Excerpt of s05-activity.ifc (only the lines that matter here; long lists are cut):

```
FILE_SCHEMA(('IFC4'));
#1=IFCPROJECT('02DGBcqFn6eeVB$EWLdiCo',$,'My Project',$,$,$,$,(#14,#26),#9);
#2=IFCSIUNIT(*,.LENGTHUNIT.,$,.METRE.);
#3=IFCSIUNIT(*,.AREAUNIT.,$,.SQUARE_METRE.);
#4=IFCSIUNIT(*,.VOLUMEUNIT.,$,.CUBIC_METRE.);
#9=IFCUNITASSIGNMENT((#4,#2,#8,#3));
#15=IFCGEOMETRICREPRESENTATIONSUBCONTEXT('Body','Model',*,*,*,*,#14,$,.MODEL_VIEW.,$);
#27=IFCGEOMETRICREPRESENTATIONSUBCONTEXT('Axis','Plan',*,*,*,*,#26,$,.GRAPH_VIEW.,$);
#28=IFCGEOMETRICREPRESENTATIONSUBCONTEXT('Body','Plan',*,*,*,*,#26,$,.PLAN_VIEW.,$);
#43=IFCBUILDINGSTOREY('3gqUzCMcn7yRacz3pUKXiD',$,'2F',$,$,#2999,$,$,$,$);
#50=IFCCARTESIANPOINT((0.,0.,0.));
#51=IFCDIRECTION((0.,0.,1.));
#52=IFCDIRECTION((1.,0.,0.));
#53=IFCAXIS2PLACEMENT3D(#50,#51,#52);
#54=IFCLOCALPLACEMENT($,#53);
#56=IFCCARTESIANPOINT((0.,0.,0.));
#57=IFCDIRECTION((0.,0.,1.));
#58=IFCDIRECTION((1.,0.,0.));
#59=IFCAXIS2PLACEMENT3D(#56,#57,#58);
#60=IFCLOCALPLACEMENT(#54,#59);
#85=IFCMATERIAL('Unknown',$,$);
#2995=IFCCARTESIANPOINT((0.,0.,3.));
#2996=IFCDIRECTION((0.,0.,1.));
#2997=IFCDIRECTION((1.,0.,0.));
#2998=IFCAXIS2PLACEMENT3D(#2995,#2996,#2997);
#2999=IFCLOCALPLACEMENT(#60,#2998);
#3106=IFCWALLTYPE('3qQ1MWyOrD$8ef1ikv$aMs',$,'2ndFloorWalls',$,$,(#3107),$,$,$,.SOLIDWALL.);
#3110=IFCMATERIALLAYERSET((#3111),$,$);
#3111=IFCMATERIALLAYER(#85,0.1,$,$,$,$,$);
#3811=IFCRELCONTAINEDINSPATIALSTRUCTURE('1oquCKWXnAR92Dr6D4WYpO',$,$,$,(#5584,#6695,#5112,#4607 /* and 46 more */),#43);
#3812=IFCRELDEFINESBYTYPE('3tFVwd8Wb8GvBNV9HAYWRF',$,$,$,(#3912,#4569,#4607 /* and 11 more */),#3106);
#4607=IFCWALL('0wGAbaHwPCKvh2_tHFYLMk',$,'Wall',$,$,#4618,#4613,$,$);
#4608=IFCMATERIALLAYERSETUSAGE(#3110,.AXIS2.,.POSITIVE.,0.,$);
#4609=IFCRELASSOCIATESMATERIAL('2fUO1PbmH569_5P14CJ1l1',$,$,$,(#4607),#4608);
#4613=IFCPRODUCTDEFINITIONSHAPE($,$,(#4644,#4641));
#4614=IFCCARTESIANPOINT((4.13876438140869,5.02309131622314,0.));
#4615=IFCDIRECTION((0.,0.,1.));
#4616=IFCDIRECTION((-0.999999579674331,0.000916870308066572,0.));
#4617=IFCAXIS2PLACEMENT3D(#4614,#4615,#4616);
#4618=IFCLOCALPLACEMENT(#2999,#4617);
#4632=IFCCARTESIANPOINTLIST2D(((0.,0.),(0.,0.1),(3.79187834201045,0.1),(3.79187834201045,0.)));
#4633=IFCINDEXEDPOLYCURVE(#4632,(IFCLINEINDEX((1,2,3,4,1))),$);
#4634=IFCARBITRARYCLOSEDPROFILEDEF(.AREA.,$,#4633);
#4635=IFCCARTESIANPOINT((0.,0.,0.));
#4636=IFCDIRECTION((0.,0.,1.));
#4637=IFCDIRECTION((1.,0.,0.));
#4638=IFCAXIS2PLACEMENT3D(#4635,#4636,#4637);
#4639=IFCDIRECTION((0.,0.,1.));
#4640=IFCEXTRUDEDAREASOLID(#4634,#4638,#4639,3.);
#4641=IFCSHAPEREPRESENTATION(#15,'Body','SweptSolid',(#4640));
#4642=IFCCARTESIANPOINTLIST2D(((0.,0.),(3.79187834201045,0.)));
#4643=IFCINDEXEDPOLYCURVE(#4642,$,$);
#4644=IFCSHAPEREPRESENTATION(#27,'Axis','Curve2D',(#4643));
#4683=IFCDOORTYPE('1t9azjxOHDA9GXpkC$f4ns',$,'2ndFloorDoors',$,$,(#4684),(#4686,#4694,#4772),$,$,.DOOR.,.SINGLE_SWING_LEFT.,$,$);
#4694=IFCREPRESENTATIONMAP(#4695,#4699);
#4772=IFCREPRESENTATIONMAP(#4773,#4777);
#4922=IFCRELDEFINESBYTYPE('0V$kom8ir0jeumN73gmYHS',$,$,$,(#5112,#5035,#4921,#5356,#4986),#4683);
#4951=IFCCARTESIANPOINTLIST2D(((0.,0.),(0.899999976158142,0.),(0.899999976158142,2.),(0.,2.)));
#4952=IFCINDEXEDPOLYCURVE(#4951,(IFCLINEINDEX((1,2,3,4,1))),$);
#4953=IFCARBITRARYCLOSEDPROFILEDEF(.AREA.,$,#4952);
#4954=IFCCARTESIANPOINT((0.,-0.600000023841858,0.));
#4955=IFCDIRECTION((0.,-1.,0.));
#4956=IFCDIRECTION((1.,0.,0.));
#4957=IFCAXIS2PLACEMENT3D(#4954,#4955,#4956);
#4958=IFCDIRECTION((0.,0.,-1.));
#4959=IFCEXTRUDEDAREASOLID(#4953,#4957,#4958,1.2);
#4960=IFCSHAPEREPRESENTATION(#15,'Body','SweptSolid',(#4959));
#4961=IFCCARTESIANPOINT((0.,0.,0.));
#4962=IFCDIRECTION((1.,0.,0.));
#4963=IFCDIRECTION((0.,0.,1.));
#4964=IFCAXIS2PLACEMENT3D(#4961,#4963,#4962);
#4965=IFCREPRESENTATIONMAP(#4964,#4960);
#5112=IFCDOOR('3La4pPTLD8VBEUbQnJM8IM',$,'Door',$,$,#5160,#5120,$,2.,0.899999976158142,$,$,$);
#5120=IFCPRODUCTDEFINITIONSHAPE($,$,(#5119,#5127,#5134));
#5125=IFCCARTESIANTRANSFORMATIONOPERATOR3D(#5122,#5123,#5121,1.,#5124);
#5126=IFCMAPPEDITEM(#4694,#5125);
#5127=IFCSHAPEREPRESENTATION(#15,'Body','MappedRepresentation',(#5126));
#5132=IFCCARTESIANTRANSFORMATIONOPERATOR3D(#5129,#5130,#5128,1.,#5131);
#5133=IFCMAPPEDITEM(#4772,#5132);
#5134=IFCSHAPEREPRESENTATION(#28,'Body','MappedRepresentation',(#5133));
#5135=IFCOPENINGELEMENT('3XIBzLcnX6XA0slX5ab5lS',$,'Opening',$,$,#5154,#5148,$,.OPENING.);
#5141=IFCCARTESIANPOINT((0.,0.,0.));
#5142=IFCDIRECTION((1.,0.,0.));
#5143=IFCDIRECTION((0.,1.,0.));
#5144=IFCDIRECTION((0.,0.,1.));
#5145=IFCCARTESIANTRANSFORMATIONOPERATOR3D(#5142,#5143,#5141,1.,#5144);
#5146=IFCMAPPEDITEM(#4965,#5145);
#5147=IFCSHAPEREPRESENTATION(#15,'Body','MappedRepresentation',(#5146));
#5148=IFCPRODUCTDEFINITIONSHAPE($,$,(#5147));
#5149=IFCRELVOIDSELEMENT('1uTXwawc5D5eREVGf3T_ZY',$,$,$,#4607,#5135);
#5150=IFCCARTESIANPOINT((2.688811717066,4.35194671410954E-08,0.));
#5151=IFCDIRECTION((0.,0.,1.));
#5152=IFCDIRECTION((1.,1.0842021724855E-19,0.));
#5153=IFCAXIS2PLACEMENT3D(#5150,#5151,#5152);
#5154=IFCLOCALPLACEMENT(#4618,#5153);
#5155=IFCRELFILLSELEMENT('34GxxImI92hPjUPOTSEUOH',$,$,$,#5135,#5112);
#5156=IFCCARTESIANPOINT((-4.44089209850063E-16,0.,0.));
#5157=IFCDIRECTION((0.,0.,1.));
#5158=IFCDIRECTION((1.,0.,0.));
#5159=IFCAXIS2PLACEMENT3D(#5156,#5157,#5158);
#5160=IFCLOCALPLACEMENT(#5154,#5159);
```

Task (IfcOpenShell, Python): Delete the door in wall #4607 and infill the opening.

```python
import ifcopenshell
import ifcopenshell.api.feature
import ifcopenshell.api.root
import ifcopenshell.geom
import ifcopenshell.util.shape

model = ifcopenshell.open("s05-activity.ifc")
settings = ifcopenshell.geom.settings()


def volume(element):
    """Net volume in cubic metres, openings subtracted."""
    shape = ifcopenshell.geom.create_shape(settings, element)
    return ifcopenshell.util.shape.get_volume(shape.geometry)


door = model.by_guid("3La4pPTLD8VBEUbQnJM8IM")
opening = door.FillsVoids[0].RelatingOpeningElement
wall = opening.VoidsElements[0].RelatingBuildingElement
before = volume(wall)

ifcopenshell.api.root.remove_product(model, product=door)
ifcopenshell.api.feature.remove_feature(model, feature=opening)

after = volume(wall)

print(f"wall volume {before:.3f} -> {after:.3f} m3")

model.write("s05-activity_rev.ifc")
```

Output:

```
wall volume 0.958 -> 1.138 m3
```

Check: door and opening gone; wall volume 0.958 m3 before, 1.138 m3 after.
